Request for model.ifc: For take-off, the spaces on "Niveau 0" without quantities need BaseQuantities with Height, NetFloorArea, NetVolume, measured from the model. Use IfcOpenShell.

First a look at what the model holds.

```python
import ifcopenshell
import ifcopenshell.util.element
import ifcopenshell.util.unit

model = ifcopenshell.open("model.ifc")
print(model.schema)
for unit_type in ("LENGTHUNIT", "AREAUNIT", "VOLUMEUNIT"):
    print(unit_type, ifcopenshell.util.unit.calculate_unit_scale(model, unit_type))
storey = next(s for s in model.by_type("IfcBuildingStorey") if s.Name == "Niveau 0")
spaces = [e for e in ifcopenshell.util.element.get_decomposition(storey) if e.is_a("IfcSpace")]
for e in sorted(spaces, key=lambda e: e.id()):
    print(e.id(), e.is_a(), e.Name, list(ifcopenshell.util.element.get_psets(e, qtos_only=True)), sep=" | ")
```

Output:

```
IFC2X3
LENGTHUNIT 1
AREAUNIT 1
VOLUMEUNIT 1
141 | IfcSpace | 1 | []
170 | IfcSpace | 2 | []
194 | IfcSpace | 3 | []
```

```python
import ifcopenshell
import ifcopenshell.api.pset
import ifcopenshell.geom
import ifcopenshell.util.element
import ifcopenshell.util.shape
import ifcopenshell.util.unit

model = ifcopenshell.open("model.ifc")
unit_scale = ifcopenshell.util.unit.calculate_unit_scale(model)
area_scale = ifcopenshell.util.unit.calculate_unit_scale(model, "AREAUNIT")
volume_scale = ifcopenshell.util.unit.calculate_unit_scale(model, "VOLUMEUNIT")
settings = ifcopenshell.geom.settings()

storey = next(s for s in model.by_type("IfcBuildingStorey") if s.Name == "Niveau 0")
spaces = [e for e in ifcopenshell.util.element.get_decomposition(storey) if e.is_a("IfcSpace")]

for e in sorted(spaces, key=lambda e: e.id()):
    if ifcopenshell.util.element.get_psets(e, qtos_only=True, should_inherit=False):
        continue
    # Geometry comes back in metres, in the element's own axes.
    shape = ifcopenshell.geom.create_shape(settings, e)
    values = {
        "Height": ifcopenshell.util.shape.get_z(shape.geometry) / unit_scale,
        "NetFloorArea": ifcopenshell.util.shape.get_footprint_area(shape.geometry) / area_scale,
        "NetVolume": ifcopenshell.util.shape.get_volume(shape.geometry) / volume_scale,
    }
    qto = ifcopenshell.api.pset.add_qto(model, product=e, name="BaseQuantities")
    ifcopenshell.api.pset.edit_qto(model, qto=qto, properties=values)
    print(e.id(), {k: round(v, 3) for k, v in values.items()})

model.write("model-out.ifc")
```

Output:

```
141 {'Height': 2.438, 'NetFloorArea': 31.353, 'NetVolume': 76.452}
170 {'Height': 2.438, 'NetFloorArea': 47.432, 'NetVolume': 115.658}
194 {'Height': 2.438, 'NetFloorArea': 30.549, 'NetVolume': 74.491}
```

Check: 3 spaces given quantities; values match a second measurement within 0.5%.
